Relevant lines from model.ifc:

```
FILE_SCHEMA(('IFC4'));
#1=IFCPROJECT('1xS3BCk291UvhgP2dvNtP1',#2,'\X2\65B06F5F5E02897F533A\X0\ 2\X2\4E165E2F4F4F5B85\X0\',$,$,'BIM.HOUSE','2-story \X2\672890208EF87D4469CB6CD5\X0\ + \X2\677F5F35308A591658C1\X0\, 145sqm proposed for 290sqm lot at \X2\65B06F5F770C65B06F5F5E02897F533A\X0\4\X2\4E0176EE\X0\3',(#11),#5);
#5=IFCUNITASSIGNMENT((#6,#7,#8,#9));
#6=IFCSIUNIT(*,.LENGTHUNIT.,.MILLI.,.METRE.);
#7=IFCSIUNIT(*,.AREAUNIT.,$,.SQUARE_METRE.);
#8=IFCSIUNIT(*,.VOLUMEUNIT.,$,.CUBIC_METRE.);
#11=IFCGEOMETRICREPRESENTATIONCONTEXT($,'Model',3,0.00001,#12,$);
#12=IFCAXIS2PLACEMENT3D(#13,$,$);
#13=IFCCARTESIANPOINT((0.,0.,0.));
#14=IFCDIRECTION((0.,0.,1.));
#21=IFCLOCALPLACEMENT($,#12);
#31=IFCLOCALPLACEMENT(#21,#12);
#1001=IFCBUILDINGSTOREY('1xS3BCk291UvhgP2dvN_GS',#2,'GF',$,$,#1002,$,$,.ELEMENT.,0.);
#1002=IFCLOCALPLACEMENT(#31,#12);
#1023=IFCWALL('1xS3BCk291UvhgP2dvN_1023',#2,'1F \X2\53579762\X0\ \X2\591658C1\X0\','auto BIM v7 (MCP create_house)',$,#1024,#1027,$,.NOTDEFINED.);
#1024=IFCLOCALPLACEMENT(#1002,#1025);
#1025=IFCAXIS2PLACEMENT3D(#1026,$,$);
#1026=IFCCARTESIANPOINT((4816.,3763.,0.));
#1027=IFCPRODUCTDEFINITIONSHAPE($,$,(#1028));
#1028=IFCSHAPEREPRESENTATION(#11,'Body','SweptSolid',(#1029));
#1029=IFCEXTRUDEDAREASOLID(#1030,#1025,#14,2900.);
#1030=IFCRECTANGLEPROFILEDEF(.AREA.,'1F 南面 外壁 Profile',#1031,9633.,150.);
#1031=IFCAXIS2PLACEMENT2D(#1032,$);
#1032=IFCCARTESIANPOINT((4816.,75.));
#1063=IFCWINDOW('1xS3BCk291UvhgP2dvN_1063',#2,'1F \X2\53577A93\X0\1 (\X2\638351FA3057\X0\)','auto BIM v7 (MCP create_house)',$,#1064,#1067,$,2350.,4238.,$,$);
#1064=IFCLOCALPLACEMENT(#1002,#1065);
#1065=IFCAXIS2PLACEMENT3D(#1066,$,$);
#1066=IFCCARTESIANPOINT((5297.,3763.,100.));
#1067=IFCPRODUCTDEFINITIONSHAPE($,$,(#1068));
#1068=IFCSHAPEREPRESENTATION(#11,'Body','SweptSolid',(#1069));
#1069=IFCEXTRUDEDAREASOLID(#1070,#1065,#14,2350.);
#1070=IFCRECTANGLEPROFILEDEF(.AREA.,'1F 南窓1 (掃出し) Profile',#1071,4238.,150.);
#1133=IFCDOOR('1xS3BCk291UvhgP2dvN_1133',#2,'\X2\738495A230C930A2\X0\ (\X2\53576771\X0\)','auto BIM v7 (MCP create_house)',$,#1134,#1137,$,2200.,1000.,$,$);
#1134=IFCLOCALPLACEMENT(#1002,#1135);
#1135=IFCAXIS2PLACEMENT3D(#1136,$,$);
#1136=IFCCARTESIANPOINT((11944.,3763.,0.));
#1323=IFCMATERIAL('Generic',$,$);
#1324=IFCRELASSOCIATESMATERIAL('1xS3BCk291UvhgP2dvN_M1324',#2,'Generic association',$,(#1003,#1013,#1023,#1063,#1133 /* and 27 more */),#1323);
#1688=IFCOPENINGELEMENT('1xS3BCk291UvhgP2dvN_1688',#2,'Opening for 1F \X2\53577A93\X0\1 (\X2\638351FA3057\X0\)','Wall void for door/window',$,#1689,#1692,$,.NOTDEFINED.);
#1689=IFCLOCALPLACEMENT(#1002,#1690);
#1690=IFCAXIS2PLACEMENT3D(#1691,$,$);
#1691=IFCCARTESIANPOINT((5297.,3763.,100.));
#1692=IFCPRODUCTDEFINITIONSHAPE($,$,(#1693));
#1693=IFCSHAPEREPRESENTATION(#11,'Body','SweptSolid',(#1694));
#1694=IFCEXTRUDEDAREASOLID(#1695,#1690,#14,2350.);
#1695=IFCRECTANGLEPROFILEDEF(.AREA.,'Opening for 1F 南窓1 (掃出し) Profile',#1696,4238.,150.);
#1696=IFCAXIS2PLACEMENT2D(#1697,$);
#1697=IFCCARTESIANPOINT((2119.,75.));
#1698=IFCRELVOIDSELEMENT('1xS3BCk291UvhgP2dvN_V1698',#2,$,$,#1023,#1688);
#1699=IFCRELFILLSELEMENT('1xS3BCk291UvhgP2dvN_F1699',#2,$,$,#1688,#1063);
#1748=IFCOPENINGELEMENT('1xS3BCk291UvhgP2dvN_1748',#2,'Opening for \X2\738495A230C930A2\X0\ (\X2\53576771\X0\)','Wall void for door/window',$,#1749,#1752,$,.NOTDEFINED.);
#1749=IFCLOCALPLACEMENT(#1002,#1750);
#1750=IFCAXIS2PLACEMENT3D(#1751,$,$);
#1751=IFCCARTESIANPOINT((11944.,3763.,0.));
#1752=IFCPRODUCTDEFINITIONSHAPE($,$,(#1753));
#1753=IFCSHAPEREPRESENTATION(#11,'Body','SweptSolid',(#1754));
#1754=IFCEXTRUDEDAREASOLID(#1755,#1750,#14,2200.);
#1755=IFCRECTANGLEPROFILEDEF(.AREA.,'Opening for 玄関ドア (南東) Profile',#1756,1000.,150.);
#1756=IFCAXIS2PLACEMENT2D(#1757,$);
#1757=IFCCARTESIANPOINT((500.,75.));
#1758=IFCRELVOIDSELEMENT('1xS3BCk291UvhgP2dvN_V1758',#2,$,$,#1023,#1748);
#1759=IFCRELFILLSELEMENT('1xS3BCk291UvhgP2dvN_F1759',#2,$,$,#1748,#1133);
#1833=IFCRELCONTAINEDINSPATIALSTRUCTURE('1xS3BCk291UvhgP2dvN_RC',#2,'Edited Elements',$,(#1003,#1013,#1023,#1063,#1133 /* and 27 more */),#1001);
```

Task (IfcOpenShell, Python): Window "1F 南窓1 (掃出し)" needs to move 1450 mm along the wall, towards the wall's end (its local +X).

```python
import ifcopenshell
import ifcopenshell.api.geometry
import ifcopenshell.util.placement
import ifcopenshell.util.unit

model = ifcopenshell.open("model.ifc")
unit_scale = ifcopenshell.util.unit.calculate_unit_scale(model)

window = model.by_guid("1xS3BCk291UvhgP2dvN_1063")
opening = window.FillsVoids[0].RelatingOpeningElement
wall = opening.VoidsElements[0].RelatingBuildingElement

wall_matrix = ifcopenshell.util.placement.get_local_placement(wall.ObjectPlacement)
shift = wall_matrix[:3, 0] * 1.45 / unit_scale
before = ifcopenshell.util.placement.get_local_placement(window.ObjectPlacement)[:3, 3].copy()

# The window is not placed relative to its opening, so move both.
for product in (opening, window):
    matrix = ifcopenshell.util.placement.get_local_placement(product.ObjectPlacement)
    matrix[:3, 3] += shift
    ifcopenshell.api.geometry.edit_object_placement(model, product=product, matrix=matrix, is_si=False)

after = ifcopenshell.util.placement.get_local_placement(window.ObjectPlacement)[:3, 3]
print("window moved by", (after - before).round(3) + 0.0)

model.write("model_v2.ifc")
```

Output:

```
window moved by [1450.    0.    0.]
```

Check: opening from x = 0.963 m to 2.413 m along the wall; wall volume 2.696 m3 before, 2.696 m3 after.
